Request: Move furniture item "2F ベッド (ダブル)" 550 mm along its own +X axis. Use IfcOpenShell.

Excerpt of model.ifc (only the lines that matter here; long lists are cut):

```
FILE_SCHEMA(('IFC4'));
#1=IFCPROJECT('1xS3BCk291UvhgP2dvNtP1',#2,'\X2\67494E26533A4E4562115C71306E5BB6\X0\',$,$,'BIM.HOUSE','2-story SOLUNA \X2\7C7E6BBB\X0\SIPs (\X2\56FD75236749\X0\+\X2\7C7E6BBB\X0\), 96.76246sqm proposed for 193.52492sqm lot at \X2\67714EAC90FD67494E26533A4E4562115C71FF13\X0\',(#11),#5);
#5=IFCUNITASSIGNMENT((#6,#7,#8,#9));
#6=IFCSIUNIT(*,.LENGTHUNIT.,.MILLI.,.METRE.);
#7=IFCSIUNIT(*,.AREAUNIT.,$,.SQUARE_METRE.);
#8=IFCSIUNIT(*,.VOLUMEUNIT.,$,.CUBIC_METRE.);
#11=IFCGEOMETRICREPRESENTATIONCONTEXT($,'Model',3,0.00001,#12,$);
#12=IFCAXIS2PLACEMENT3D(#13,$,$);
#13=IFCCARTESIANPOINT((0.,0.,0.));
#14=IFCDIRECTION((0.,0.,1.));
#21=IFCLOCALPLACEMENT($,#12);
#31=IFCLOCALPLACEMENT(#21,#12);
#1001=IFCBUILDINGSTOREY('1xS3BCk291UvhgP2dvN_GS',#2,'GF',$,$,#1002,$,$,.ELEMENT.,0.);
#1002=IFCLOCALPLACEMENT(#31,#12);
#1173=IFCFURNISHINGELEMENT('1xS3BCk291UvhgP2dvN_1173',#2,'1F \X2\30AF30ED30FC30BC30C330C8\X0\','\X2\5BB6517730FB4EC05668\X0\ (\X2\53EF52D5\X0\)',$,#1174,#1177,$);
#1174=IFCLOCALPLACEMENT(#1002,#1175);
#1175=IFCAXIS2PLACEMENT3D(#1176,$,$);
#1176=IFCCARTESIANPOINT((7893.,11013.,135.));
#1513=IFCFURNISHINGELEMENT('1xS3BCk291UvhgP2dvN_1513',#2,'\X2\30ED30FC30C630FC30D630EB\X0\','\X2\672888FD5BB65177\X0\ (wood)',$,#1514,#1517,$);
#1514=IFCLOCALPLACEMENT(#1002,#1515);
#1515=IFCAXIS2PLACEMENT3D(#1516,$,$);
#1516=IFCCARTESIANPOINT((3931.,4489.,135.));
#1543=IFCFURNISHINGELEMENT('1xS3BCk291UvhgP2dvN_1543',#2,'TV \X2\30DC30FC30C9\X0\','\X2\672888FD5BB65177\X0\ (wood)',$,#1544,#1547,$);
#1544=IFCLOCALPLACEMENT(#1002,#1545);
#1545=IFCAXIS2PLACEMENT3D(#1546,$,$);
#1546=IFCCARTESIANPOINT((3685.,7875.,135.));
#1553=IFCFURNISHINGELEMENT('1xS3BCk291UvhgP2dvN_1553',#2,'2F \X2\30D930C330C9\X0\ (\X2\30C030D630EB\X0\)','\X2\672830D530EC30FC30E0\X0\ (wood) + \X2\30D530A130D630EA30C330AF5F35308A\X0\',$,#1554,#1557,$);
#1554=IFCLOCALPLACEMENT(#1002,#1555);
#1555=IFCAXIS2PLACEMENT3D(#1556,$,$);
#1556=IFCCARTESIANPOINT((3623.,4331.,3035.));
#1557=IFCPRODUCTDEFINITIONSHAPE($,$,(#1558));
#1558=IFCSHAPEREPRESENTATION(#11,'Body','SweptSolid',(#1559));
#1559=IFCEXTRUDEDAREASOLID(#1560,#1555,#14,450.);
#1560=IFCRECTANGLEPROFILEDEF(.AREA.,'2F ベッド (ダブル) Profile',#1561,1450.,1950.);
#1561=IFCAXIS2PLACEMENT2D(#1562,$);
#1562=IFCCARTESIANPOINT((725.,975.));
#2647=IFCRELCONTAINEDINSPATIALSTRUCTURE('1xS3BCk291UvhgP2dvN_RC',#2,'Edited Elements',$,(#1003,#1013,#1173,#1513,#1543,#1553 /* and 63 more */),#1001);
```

```python
import ifcopenshell
import ifcopenshell.api.geometry
import ifcopenshell.util.placement
import ifcopenshell.util.unit

model = ifcopenshell.open("model.ifc")
unit_scale = ifcopenshell.util.unit.calculate_unit_scale(model)

item = model.by_id(1553)
matrix = ifcopenshell.util.placement.get_local_placement(item.ObjectPlacement)
matrix[:3, 3] += matrix[:3, 0] * 0.55 / unit_scale
ifcopenshell.api.geometry.edit_object_placement(model, product=item, matrix=matrix, is_si=False)

print(ifcopenshell.util.placement.get_local_placement(item.ObjectPlacement).round(3) + 0.0)

model.write("model_edited.ifc")
```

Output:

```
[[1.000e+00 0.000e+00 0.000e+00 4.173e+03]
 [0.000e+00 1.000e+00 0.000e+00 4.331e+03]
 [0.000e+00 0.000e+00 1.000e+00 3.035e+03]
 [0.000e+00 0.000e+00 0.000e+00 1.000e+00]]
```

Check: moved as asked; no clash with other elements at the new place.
